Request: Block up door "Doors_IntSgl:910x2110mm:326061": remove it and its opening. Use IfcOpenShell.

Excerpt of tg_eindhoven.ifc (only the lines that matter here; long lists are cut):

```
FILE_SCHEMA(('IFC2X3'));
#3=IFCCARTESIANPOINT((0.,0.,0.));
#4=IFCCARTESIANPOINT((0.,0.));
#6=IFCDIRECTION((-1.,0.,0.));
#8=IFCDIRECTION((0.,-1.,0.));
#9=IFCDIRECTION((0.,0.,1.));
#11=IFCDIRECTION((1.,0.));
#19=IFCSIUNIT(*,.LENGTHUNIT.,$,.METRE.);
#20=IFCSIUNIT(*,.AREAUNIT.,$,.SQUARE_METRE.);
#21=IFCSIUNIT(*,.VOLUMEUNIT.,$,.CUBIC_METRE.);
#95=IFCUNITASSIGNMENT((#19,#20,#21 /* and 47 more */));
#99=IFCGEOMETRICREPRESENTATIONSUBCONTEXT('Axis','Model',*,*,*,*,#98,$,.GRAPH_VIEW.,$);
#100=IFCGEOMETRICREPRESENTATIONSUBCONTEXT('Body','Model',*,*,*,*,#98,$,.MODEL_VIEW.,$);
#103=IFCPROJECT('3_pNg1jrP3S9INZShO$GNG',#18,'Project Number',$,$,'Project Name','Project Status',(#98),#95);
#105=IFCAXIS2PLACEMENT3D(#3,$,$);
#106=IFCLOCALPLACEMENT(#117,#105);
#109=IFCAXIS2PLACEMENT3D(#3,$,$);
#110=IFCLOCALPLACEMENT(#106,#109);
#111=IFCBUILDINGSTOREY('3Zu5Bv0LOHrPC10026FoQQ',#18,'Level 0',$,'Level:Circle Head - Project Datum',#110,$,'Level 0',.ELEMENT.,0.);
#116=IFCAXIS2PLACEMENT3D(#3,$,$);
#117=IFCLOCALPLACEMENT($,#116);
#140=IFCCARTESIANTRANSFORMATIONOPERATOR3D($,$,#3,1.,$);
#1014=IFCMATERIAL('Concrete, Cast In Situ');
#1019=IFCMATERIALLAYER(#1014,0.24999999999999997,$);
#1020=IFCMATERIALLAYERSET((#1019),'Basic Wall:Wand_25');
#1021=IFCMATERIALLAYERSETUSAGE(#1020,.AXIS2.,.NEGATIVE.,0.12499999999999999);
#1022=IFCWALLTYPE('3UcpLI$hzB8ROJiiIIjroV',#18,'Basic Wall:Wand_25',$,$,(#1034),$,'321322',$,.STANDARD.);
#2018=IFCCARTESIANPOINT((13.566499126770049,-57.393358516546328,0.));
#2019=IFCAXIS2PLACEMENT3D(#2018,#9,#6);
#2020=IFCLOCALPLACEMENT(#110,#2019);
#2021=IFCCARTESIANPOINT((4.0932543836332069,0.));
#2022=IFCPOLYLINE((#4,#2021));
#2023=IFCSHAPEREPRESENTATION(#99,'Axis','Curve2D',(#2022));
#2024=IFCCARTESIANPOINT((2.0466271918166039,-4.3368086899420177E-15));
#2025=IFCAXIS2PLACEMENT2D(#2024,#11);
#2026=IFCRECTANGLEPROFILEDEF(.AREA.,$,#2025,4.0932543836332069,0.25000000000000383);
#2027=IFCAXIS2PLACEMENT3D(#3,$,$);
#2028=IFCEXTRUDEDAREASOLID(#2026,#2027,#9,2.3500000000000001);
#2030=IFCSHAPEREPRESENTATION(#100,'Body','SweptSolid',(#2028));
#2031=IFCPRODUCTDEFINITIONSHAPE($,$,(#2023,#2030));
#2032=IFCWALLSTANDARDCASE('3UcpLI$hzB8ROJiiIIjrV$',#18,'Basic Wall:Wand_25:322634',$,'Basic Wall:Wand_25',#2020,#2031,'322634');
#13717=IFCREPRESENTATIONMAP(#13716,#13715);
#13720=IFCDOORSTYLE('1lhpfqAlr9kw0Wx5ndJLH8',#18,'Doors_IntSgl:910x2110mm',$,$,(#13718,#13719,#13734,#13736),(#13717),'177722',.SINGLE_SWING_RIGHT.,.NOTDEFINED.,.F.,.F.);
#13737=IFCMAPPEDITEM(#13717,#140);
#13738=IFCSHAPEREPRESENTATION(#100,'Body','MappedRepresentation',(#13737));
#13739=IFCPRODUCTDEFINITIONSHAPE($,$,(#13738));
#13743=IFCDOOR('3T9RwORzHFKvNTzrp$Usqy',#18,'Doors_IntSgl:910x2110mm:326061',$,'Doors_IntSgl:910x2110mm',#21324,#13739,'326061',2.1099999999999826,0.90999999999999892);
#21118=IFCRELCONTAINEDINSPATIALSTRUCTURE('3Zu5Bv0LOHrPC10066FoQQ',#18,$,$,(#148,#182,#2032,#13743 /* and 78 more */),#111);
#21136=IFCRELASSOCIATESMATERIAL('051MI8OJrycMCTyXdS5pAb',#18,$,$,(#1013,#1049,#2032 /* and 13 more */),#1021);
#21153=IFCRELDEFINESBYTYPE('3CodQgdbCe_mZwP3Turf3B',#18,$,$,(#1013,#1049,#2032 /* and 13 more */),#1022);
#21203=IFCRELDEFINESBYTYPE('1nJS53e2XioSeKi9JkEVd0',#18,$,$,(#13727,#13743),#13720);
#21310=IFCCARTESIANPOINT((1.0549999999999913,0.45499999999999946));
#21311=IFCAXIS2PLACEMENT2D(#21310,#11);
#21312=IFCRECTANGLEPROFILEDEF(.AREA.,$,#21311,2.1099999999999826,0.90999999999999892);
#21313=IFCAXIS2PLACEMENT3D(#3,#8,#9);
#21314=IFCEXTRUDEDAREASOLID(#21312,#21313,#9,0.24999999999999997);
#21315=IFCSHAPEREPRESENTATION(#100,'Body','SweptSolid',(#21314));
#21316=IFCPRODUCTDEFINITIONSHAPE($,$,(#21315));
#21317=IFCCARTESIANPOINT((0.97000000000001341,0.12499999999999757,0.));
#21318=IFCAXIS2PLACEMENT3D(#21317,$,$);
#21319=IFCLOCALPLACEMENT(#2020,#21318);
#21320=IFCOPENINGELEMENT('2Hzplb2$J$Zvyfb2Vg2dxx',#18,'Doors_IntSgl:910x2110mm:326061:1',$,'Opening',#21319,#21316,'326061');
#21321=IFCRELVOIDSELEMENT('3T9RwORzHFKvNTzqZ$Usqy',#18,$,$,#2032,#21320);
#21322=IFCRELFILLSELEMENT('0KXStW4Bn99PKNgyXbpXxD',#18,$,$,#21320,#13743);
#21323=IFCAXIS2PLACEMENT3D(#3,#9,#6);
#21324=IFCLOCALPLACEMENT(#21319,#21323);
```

```python
import ifcopenshell
import ifcopenshell.api.feature
import ifcopenshell.api.root
import ifcopenshell.geom
import ifcopenshell.util.shape

model = ifcopenshell.open("tg_eindhoven.ifc")
settings = ifcopenshell.geom.settings()


def volume(element):
    """Net volume in cubic metres, openings subtracted."""
    shape = ifcopenshell.geom.create_shape(settings, element)
    return ifcopenshell.util.shape.get_volume(shape.geometry)


door = model.by_guid("3T9RwORzHFKvNTzrp$Usqy")
opening = door.FillsVoids[0].RelatingOpeningElement
wall = opening.VoidsElements[0].RelatingBuildingElement
before = volume(wall)

ifcopenshell.api.root.remove_product(model, product=door)
ifcopenshell.api.feature.remove_feature(model, feature=opening)

after = volume(wall)

print(f"wall volume {before:.3f} -> {after:.3f} m3")

model.write("tg_eindhoven-out.ifc")
```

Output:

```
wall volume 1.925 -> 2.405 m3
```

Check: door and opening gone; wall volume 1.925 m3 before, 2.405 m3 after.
